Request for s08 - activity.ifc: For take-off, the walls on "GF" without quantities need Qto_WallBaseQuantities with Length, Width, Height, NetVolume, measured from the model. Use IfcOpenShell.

First a look at what the model holds.

```python
import ifcopenshell
import ifcopenshell.util.element
import ifcopenshell.util.unit

model = ifcopenshell.open("s08 - activity.ifc")
print(model.schema)
for unit_type in ("LENGTHUNIT", "AREAUNIT", "VOLUMEUNIT"):
    print(unit_type, ifcopenshell.util.unit.calculate_unit_scale(model, unit_type))
storey = next(s for s in model.by_type("IfcBuildingStorey") if s.Name == "GF")
walls = [e for e in ifcopenshell.util.element.get_decomposition(storey) if e.is_a("IfcWall")]
for e in sorted(walls, key=lambda e: e.id()):
    print(e.id(), e.is_a(), e.Name, list(ifcopenshell.util.element.get_psets(e, qtos_only=True)), sep=" | ")
```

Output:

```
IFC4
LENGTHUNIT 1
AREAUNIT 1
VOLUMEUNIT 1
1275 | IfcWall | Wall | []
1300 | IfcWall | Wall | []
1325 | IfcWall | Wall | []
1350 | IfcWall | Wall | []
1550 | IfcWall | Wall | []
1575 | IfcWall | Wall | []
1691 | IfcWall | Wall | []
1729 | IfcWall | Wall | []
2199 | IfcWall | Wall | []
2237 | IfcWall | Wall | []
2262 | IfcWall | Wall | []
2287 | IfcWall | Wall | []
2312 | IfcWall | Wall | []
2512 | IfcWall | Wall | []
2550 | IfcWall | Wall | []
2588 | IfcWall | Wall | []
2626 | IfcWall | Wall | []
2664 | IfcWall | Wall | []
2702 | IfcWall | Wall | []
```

```python
import ifcopenshell
import ifcopenshell.api.pset
import ifcopenshell.geom
import ifcopenshell.util.element
import ifcopenshell.util.shape
import ifcopenshell.util.unit

model = ifcopenshell.open("s08 - activity.ifc")
unit_scale = ifcopenshell.util.unit.calculate_unit_scale(model)
volume_scale = ifcopenshell.util.unit.calculate_unit_scale(model, "VOLUMEUNIT")
settings = ifcopenshell.geom.settings()

storey = next(s for s in model.by_type("IfcBuildingStorey") if s.Name == "GF")
walls = [e for e in ifcopenshell.util.element.get_decomposition(storey) if e.is_a("IfcWall")]

for e in sorted(walls, key=lambda e: e.id()):
    if ifcopenshell.util.element.get_psets(e, qtos_only=True, should_inherit=False):
        continue
    # Geometry comes back in metres, in the element's own axes.
    shape = ifcopenshell.geom.create_shape(settings, e)
    values = {
        "Length": ifcopenshell.util.shape.get_x(shape.geometry) / unit_scale,
        "Width": ifcopenshell.util.shape.get_y(shape.geometry) / unit_scale,
        "Height": ifcopenshell.util.shape.get_z(shape.geometry) / unit_scale,
        "NetVolume": ifcopenshell.util.shape.get_volume(shape.geometry) / volume_scale,
    }
    qto = ifcopenshell.api.pset.add_qto(model, product=e, name="Qto_WallBaseQuantities")
    ifcopenshell.api.pset.edit_qto(model, qto=qto, properties=values)
    print(e.id(), {k: round(v, 3) for k, v in values.items()})

model.write("s08 - activity_v2.ifc")
```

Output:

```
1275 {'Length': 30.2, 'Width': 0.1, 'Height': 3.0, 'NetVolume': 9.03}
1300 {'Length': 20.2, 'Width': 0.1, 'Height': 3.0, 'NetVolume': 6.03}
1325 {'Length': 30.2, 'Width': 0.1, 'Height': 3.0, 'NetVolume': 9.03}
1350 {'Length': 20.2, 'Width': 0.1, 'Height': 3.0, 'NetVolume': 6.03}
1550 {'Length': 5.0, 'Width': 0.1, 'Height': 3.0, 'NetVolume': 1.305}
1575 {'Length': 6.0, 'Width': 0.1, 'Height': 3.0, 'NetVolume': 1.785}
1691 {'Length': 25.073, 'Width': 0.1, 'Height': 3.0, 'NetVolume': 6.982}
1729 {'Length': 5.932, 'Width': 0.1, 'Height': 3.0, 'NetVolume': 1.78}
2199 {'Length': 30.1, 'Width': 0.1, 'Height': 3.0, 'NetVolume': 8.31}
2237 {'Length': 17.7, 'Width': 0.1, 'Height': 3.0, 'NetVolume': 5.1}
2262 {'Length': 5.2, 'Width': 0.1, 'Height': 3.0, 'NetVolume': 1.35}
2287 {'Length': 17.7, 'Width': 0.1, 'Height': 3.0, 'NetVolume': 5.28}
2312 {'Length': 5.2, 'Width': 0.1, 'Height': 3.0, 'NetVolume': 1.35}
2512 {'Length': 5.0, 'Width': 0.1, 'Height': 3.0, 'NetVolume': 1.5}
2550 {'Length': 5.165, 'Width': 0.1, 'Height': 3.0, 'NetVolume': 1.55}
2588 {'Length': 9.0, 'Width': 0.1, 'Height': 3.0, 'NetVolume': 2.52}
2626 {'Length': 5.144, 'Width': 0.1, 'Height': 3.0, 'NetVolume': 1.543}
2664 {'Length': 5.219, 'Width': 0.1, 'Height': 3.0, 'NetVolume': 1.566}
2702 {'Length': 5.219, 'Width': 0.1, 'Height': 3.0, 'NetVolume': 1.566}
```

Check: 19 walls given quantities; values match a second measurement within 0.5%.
